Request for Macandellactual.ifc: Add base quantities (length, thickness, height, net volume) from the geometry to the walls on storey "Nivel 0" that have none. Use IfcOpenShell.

First a look at what the model holds.

```python
import ifcopenshell
import ifcopenshell.util.element
import ifcopenshell.util.unit

model = ifcopenshell.open("Macandellactual.ifc")
print(model.schema)
for unit_type in ("LENGTHUNIT", "AREAUNIT", "VOLUMEUNIT"):
    print(unit_type, ifcopenshell.util.unit.calculate_unit_scale(model, unit_type))
storey = next(s for s in model.by_type("IfcBuildingStorey") if s.Name == "Nivel 0")
walls = [e for e in ifcopenshell.util.element.get_decomposition(storey) if e.is_a("IfcWall")]
for e in sorted(walls, key=lambda e: e.id()):
    print(e.id(), e.is_a(), e.Name, list(ifcopenshell.util.element.get_psets(e, qtos_only=True)), sep=" | ")
```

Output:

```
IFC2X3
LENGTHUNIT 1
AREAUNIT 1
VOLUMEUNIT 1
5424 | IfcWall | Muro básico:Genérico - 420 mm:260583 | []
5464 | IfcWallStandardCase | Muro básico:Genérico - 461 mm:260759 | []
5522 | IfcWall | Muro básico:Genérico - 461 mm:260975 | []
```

```python
import ifcopenshell
import ifcopenshell.api.pset
import ifcopenshell.geom
import ifcopenshell.util.element
import ifcopenshell.util.shape
import ifcopenshell.util.unit

model = ifcopenshell.open("Macandellactual.ifc")
unit_scale = ifcopenshell.util.unit.calculate_unit_scale(model)
volume_scale = ifcopenshell.util.unit.calculate_unit_scale(model, "VOLUMEUNIT")
settings = ifcopenshell.geom.settings()

storey = next(s for s in model.by_type("IfcBuildingStorey") if s.Name == "Nivel 0")
walls = [e for e in ifcopenshell.util.element.get_decomposition(storey) if e.is_a("IfcWall")]

for e in sorted(walls, key=lambda e: e.id()):
    if ifcopenshell.util.element.get_psets(e, qtos_only=True, should_inherit=False):
        continue
    # Geometry comes back in metres, in the element's own axes.
    shape = ifcopenshell.geom.create_shape(settings, e)
    values = {
        "Length": ifcopenshell.util.shape.get_x(shape.geometry) / unit_scale,
        "Width": ifcopenshell.util.shape.get_y(shape.geometry) / unit_scale,
        "Height": ifcopenshell.util.shape.get_z(shape.geometry) / unit_scale,
        "NetVolume": ifcopenshell.util.shape.get_volume(shape.geometry) / volume_scale,
    }
    qto = ifcopenshell.api.pset.add_qto(model, product=e, name="BaseQuantities")
    ifcopenshell.api.pset.edit_qto(model, qto=qto, properties=values)
    print(e.id(), {k: round(v, 3) for k, v in values.items()})

model.write("Macandellactual_v2.ifc")
```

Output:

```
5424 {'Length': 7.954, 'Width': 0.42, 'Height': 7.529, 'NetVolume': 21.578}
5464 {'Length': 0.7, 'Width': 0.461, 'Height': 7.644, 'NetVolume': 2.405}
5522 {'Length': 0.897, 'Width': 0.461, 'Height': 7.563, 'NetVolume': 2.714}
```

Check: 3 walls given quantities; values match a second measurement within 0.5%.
